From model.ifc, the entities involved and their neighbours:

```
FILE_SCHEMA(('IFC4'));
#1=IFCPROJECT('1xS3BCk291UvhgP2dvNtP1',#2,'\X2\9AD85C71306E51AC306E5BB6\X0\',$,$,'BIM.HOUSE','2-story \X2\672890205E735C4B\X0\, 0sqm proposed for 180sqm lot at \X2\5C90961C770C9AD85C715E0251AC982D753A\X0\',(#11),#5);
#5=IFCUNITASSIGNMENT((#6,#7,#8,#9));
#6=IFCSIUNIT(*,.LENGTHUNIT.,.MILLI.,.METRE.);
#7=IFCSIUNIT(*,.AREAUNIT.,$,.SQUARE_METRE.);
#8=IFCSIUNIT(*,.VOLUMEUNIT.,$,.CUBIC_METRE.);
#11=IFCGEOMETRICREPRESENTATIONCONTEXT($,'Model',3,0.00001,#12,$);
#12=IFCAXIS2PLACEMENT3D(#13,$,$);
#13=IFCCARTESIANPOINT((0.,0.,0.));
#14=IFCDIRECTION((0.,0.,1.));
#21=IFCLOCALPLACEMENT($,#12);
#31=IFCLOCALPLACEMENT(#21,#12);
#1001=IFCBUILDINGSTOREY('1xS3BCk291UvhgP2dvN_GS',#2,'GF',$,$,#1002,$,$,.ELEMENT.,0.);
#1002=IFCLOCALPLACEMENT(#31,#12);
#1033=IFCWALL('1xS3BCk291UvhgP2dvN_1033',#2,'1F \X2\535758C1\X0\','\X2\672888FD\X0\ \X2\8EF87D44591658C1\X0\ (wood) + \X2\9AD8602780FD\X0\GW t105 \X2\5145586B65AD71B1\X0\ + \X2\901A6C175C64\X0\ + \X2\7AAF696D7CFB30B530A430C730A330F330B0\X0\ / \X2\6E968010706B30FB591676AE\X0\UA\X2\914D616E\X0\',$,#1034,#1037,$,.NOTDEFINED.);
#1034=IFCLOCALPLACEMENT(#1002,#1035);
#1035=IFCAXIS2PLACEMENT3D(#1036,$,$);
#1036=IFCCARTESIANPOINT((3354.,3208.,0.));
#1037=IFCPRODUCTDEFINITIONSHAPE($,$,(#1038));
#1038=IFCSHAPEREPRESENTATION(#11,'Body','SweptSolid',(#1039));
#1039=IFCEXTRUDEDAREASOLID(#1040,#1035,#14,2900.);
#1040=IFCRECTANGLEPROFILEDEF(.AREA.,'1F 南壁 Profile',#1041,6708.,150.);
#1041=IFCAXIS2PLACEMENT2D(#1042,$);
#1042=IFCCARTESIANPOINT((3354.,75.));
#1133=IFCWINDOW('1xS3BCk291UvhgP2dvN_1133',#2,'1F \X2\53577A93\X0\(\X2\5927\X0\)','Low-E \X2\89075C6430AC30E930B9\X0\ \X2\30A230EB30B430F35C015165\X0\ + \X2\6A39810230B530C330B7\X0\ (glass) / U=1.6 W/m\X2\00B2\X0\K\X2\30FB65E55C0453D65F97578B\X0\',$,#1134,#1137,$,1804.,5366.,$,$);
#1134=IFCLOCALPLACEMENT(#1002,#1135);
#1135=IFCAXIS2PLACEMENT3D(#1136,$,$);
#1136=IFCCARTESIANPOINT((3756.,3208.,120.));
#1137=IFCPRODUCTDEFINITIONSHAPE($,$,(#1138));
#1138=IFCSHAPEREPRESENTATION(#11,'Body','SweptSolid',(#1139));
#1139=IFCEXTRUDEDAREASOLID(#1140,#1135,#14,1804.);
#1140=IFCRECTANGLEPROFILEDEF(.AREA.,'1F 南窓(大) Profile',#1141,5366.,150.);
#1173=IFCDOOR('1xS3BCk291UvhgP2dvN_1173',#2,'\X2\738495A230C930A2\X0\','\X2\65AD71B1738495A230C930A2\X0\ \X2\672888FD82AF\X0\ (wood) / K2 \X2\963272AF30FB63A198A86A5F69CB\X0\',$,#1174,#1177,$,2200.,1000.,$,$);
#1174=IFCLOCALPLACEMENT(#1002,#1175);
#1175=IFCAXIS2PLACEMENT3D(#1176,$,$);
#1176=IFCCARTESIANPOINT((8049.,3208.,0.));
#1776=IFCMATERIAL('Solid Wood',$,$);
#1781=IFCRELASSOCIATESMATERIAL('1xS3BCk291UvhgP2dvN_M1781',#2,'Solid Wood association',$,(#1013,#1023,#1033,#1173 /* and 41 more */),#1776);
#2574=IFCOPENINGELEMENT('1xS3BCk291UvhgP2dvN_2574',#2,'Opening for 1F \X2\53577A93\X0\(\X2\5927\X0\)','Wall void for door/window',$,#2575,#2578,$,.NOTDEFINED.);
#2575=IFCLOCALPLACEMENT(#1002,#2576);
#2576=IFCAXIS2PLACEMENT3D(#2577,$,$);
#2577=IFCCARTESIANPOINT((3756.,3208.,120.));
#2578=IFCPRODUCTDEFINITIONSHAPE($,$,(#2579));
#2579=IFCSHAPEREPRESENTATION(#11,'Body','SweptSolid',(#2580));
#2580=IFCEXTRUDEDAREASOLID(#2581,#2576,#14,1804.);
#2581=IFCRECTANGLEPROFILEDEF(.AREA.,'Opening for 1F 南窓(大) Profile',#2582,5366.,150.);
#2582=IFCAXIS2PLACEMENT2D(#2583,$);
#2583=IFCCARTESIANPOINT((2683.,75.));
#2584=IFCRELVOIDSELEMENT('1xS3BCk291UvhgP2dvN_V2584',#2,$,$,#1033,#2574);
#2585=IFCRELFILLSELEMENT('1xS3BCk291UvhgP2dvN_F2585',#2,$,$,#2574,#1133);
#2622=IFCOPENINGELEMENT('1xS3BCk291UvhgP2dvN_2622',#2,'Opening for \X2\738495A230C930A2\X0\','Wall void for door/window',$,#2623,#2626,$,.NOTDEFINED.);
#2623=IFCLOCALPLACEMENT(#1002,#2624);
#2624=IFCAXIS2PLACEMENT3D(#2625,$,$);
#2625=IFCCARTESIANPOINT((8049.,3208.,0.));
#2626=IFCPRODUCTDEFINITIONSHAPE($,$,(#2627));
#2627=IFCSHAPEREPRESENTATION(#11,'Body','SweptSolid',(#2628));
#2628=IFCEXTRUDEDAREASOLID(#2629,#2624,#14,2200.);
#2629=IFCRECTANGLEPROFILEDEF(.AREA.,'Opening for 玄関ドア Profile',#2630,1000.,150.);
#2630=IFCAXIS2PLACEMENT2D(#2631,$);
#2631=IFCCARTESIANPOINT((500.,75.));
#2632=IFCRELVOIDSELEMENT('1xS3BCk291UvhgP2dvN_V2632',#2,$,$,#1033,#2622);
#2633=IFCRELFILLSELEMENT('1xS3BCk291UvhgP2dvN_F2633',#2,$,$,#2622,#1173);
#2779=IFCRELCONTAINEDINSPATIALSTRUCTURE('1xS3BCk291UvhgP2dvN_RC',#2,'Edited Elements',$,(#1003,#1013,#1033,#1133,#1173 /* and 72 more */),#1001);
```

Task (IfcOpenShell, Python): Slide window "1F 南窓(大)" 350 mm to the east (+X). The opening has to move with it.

```python
import ifcopenshell
import ifcopenshell.api.geometry
import ifcopenshell.util.placement

model = ifcopenshell.open("model.ifc")

window = model.by_guid("1xS3BCk291UvhgP2dvN_1133")
opening = window.FillsVoids[0].RelatingOpeningElement
wall = opening.VoidsElements[0].RelatingBuildingElement

wall_matrix = ifcopenshell.util.placement.get_local_placement(wall.ObjectPlacement)
shift = wall_matrix[:3, 0] * 350.0
before = ifcopenshell.util.placement.get_local_placement(window.ObjectPlacement)[:3, 3].copy()

# The window is not placed relative to its opening, so move both.
for product in (opening, window):
    matrix = ifcopenshell.util.placement.get_local_placement(product.ObjectPlacement)
    matrix[:3, 3] += shift
    ifcopenshell.api.geometry.edit_object_placement(model, product=product, matrix=matrix, is_si=False)

after = ifcopenshell.util.placement.get_local_placement(window.ObjectPlacement)[:3, 3]
print("window moved by", (after - before).round(3) + 0.0)

model.write("model_rev.ifc")
```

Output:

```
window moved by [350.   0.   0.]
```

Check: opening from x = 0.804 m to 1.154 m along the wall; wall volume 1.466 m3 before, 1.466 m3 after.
